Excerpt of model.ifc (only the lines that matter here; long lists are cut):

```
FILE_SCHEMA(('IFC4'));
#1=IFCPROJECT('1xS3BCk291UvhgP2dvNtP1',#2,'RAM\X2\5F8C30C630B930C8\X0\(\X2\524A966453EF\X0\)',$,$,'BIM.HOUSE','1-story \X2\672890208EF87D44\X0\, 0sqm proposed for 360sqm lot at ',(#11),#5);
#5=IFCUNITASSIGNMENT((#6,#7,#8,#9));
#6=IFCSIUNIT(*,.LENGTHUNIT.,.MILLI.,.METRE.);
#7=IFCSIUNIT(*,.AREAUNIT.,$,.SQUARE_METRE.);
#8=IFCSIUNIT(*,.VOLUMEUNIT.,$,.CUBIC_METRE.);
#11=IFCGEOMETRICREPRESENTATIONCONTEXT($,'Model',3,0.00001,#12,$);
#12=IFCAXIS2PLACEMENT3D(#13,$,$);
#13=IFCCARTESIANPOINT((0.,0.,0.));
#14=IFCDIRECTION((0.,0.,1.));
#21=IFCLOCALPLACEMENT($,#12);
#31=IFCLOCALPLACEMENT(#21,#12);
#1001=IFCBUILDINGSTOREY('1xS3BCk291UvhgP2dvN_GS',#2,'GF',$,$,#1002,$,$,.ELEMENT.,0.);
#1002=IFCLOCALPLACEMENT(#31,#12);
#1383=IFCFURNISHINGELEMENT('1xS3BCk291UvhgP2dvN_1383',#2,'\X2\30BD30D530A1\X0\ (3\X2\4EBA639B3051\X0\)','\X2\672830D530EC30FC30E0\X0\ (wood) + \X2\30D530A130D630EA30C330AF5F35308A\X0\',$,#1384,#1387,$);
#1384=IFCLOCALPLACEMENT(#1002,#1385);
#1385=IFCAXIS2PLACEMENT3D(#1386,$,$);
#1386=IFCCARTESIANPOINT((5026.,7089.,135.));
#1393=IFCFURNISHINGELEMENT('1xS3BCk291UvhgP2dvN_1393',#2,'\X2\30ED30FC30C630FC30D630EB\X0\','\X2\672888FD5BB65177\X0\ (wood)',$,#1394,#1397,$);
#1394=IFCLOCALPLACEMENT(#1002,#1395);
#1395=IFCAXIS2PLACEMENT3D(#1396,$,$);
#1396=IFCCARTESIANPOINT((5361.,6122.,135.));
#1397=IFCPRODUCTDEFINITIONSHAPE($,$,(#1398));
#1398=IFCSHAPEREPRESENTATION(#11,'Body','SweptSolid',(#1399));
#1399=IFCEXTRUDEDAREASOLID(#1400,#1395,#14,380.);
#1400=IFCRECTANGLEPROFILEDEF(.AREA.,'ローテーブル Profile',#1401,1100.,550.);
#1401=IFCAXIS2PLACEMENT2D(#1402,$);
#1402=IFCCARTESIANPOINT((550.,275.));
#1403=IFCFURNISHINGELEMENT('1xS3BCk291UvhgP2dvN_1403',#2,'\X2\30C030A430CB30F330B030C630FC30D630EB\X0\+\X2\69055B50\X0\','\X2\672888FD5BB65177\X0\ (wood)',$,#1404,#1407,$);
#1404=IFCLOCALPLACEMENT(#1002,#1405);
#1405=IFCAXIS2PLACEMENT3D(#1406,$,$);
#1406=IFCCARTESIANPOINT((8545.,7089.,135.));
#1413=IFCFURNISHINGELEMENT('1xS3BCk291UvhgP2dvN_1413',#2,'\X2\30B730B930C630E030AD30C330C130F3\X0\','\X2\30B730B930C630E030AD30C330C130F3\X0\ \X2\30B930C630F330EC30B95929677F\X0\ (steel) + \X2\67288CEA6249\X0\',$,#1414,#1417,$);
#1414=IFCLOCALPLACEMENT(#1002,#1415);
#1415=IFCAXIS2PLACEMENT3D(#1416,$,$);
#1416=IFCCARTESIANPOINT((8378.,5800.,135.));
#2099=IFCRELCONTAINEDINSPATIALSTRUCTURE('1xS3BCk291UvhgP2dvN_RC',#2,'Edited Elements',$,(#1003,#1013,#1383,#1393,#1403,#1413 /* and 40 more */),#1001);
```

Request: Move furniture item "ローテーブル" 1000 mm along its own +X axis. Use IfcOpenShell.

```python
import ifcopenshell
import ifcopenshell.api.geometry
import ifcopenshell.util.placement

model = ifcopenshell.open("model.ifc")

item = model.by_id(1393)
matrix = ifcopenshell.util.placement.get_local_placement(item.ObjectPlacement)
matrix[:3, 3] += matrix[:3, 0] * 1000.0
ifcopenshell.api.geometry.edit_object_placement(model, product=item, matrix=matrix, is_si=False)

print(ifcopenshell.util.placement.get_local_placement(item.ObjectPlacement).round(3) + 0.0)

model.write("model_v2.ifc")
```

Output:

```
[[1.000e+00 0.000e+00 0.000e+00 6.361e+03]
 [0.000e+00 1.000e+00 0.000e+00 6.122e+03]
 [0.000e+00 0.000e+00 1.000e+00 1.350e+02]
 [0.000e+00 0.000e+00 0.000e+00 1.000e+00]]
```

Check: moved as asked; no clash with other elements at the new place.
